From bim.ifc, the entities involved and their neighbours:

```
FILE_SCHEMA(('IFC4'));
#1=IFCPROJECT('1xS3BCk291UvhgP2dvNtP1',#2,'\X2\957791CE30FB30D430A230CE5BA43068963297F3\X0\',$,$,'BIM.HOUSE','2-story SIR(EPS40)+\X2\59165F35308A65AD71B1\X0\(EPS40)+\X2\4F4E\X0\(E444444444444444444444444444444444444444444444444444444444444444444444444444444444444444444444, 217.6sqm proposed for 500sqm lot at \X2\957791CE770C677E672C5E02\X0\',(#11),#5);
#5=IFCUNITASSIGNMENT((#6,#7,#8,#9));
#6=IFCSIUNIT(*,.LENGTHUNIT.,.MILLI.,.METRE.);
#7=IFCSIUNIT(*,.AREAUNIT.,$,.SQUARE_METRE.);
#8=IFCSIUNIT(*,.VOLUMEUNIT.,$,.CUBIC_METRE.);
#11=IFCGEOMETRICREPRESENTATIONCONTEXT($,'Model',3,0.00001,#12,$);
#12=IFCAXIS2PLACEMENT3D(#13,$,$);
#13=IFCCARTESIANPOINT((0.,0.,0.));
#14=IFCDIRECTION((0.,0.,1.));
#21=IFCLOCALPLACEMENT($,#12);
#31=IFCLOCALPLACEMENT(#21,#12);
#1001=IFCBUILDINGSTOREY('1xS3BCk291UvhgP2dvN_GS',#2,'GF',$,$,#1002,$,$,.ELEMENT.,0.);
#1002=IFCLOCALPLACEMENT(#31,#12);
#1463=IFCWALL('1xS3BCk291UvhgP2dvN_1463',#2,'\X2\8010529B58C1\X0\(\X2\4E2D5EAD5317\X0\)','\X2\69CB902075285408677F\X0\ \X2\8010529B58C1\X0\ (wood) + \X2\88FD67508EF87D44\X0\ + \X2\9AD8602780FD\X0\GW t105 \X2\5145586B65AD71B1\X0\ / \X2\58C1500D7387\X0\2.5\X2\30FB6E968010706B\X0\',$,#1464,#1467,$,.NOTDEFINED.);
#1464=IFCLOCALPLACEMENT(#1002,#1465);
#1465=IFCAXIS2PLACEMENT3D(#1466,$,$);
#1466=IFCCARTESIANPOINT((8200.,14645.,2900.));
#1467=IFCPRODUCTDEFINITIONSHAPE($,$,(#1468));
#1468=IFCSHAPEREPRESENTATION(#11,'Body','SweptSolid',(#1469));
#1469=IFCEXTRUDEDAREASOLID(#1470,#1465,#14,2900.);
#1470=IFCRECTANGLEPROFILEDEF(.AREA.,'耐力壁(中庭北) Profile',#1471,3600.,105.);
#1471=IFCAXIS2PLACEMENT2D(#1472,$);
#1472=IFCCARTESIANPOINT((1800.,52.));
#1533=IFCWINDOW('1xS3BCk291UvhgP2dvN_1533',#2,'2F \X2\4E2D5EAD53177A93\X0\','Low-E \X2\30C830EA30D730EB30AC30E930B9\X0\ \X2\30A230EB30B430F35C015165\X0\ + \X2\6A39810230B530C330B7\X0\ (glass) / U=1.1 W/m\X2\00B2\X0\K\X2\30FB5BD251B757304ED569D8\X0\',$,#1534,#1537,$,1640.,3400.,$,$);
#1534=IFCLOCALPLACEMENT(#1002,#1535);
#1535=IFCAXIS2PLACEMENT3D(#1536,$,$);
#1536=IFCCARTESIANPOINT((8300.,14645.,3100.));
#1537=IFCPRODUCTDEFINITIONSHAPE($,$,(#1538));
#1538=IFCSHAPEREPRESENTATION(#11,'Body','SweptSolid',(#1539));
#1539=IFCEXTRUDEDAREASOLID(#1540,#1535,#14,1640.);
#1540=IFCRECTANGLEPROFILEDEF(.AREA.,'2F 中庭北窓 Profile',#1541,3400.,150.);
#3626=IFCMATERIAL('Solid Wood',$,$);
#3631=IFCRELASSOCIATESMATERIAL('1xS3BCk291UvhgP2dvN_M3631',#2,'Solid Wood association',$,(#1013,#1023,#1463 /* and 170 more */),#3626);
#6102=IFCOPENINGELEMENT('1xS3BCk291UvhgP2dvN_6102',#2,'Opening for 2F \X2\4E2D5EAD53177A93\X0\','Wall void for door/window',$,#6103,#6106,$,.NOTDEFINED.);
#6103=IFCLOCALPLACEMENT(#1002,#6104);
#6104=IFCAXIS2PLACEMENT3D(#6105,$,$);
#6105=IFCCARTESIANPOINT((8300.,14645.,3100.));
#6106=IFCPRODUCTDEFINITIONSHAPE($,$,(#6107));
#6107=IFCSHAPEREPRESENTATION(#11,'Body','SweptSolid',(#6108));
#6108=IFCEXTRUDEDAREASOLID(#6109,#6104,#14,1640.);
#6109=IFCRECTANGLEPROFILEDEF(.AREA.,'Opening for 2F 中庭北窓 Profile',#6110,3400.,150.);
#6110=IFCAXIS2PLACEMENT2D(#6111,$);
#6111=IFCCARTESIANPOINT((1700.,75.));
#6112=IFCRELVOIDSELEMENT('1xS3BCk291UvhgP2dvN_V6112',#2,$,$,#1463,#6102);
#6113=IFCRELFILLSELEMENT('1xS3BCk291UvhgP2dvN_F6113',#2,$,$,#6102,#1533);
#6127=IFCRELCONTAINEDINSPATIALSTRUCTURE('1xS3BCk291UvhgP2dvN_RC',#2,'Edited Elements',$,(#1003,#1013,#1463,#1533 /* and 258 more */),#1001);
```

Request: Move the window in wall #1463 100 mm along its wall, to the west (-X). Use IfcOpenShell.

```python
import ifcopenshell
import ifcopenshell.api.geometry
import ifcopenshell.util.placement
import ifcopenshell.util.unit

model = ifcopenshell.open("bim.ifc")
unit_scale = ifcopenshell.util.unit.calculate_unit_scale(model)

window = model.by_guid("1xS3BCk291UvhgP2dvN_1533")
opening = window.FillsVoids[0].RelatingOpeningElement
wall = opening.VoidsElements[0].RelatingBuildingElement

wall_matrix = ifcopenshell.util.placement.get_local_placement(wall.ObjectPlacement)
shift = wall_matrix[:3, 0] * -0.1 / unit_scale
before = ifcopenshell.util.placement.get_local_placement(window.ObjectPlacement)[:3, 3].copy()

# The window is not placed relative to its opening, so move both.
for product in (opening, window):
    matrix = ifcopenshell.util.placement.get_local_placement(product.ObjectPlacement)
    matrix[:3, 3] += shift
    ifcopenshell.api.geometry.edit_object_placement(model, product=product, matrix=matrix, is_si=False)

after = ifcopenshell.util.placement.get_local_placement(window.ObjectPlacement)[:3, 3]
print("window moved by", (after - before).round(3) + 0.0)

model.write("bim_edited.ifc")
```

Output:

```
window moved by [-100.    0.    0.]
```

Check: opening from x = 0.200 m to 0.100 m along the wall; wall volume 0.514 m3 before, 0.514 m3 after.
